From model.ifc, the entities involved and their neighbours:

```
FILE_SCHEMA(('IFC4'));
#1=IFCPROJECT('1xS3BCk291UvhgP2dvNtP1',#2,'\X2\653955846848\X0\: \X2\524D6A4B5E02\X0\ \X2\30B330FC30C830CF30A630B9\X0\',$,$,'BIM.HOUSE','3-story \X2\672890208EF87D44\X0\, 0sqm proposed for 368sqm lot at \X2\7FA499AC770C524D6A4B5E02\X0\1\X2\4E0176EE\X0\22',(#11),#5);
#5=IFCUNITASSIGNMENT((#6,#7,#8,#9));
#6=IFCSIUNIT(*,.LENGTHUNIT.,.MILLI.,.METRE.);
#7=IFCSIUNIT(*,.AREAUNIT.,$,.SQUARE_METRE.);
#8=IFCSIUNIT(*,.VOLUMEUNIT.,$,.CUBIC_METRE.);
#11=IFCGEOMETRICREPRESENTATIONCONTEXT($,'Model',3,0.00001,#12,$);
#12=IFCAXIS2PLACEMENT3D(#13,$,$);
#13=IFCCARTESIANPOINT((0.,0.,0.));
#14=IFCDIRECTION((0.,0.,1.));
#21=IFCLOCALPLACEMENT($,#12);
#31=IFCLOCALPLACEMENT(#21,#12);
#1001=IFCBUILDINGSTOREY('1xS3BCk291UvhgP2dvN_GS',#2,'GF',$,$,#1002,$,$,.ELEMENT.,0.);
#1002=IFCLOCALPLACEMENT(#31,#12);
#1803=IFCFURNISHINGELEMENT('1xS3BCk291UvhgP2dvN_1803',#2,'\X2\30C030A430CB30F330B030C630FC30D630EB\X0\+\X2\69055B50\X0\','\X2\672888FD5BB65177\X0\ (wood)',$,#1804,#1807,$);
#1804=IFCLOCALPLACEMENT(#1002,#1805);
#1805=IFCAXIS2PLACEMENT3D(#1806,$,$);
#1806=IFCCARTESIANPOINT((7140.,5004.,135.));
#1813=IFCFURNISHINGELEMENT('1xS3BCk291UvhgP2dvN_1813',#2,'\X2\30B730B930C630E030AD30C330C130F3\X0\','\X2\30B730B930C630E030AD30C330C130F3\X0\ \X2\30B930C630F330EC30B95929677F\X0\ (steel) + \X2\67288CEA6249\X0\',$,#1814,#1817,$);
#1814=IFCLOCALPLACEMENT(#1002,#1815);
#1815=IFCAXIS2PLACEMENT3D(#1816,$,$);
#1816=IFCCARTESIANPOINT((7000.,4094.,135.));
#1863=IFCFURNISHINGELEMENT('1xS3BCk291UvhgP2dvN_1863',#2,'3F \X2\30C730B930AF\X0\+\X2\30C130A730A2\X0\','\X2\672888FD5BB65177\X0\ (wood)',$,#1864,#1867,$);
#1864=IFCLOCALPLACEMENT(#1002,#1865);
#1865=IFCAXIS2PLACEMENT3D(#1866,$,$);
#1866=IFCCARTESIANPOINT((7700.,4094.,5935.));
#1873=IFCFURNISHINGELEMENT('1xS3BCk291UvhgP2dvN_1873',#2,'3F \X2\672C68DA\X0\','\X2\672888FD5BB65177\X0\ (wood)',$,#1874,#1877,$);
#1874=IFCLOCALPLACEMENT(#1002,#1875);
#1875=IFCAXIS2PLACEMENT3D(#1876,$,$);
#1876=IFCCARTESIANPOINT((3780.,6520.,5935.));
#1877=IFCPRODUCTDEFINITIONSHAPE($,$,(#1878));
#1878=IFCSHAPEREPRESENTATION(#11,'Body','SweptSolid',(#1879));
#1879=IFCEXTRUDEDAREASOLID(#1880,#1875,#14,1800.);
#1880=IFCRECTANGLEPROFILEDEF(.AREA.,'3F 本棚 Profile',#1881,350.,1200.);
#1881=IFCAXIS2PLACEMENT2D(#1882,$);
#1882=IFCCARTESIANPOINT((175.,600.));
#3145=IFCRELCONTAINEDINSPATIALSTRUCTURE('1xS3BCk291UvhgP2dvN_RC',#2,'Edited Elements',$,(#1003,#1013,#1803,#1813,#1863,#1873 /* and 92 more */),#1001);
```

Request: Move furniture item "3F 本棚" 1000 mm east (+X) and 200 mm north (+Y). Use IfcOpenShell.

```python
import ifcopenshell
import ifcopenshell.api.geometry
import ifcopenshell.util.placement
import ifcopenshell.util.unit

model = ifcopenshell.open("model.ifc")
unit_scale = ifcopenshell.util.unit.calculate_unit_scale(model)

item = model.by_guid("1xS3BCk291UvhgP2dvN_1873")
matrix = ifcopenshell.util.placement.get_local_placement(item.ObjectPlacement)
matrix[0, 3] += 1 / unit_scale
matrix[1, 3] += 0.2 / unit_scale
ifcopenshell.api.geometry.edit_object_placement(model, product=item, matrix=matrix, is_si=False)

print(ifcopenshell.util.placement.get_local_placement(item.ObjectPlacement).round(3) + 0.0)

model.write("model_v2.ifc")
```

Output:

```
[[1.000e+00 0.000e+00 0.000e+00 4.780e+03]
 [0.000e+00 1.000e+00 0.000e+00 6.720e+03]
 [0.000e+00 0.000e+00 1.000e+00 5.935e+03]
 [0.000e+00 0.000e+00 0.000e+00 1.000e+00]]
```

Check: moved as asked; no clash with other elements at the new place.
